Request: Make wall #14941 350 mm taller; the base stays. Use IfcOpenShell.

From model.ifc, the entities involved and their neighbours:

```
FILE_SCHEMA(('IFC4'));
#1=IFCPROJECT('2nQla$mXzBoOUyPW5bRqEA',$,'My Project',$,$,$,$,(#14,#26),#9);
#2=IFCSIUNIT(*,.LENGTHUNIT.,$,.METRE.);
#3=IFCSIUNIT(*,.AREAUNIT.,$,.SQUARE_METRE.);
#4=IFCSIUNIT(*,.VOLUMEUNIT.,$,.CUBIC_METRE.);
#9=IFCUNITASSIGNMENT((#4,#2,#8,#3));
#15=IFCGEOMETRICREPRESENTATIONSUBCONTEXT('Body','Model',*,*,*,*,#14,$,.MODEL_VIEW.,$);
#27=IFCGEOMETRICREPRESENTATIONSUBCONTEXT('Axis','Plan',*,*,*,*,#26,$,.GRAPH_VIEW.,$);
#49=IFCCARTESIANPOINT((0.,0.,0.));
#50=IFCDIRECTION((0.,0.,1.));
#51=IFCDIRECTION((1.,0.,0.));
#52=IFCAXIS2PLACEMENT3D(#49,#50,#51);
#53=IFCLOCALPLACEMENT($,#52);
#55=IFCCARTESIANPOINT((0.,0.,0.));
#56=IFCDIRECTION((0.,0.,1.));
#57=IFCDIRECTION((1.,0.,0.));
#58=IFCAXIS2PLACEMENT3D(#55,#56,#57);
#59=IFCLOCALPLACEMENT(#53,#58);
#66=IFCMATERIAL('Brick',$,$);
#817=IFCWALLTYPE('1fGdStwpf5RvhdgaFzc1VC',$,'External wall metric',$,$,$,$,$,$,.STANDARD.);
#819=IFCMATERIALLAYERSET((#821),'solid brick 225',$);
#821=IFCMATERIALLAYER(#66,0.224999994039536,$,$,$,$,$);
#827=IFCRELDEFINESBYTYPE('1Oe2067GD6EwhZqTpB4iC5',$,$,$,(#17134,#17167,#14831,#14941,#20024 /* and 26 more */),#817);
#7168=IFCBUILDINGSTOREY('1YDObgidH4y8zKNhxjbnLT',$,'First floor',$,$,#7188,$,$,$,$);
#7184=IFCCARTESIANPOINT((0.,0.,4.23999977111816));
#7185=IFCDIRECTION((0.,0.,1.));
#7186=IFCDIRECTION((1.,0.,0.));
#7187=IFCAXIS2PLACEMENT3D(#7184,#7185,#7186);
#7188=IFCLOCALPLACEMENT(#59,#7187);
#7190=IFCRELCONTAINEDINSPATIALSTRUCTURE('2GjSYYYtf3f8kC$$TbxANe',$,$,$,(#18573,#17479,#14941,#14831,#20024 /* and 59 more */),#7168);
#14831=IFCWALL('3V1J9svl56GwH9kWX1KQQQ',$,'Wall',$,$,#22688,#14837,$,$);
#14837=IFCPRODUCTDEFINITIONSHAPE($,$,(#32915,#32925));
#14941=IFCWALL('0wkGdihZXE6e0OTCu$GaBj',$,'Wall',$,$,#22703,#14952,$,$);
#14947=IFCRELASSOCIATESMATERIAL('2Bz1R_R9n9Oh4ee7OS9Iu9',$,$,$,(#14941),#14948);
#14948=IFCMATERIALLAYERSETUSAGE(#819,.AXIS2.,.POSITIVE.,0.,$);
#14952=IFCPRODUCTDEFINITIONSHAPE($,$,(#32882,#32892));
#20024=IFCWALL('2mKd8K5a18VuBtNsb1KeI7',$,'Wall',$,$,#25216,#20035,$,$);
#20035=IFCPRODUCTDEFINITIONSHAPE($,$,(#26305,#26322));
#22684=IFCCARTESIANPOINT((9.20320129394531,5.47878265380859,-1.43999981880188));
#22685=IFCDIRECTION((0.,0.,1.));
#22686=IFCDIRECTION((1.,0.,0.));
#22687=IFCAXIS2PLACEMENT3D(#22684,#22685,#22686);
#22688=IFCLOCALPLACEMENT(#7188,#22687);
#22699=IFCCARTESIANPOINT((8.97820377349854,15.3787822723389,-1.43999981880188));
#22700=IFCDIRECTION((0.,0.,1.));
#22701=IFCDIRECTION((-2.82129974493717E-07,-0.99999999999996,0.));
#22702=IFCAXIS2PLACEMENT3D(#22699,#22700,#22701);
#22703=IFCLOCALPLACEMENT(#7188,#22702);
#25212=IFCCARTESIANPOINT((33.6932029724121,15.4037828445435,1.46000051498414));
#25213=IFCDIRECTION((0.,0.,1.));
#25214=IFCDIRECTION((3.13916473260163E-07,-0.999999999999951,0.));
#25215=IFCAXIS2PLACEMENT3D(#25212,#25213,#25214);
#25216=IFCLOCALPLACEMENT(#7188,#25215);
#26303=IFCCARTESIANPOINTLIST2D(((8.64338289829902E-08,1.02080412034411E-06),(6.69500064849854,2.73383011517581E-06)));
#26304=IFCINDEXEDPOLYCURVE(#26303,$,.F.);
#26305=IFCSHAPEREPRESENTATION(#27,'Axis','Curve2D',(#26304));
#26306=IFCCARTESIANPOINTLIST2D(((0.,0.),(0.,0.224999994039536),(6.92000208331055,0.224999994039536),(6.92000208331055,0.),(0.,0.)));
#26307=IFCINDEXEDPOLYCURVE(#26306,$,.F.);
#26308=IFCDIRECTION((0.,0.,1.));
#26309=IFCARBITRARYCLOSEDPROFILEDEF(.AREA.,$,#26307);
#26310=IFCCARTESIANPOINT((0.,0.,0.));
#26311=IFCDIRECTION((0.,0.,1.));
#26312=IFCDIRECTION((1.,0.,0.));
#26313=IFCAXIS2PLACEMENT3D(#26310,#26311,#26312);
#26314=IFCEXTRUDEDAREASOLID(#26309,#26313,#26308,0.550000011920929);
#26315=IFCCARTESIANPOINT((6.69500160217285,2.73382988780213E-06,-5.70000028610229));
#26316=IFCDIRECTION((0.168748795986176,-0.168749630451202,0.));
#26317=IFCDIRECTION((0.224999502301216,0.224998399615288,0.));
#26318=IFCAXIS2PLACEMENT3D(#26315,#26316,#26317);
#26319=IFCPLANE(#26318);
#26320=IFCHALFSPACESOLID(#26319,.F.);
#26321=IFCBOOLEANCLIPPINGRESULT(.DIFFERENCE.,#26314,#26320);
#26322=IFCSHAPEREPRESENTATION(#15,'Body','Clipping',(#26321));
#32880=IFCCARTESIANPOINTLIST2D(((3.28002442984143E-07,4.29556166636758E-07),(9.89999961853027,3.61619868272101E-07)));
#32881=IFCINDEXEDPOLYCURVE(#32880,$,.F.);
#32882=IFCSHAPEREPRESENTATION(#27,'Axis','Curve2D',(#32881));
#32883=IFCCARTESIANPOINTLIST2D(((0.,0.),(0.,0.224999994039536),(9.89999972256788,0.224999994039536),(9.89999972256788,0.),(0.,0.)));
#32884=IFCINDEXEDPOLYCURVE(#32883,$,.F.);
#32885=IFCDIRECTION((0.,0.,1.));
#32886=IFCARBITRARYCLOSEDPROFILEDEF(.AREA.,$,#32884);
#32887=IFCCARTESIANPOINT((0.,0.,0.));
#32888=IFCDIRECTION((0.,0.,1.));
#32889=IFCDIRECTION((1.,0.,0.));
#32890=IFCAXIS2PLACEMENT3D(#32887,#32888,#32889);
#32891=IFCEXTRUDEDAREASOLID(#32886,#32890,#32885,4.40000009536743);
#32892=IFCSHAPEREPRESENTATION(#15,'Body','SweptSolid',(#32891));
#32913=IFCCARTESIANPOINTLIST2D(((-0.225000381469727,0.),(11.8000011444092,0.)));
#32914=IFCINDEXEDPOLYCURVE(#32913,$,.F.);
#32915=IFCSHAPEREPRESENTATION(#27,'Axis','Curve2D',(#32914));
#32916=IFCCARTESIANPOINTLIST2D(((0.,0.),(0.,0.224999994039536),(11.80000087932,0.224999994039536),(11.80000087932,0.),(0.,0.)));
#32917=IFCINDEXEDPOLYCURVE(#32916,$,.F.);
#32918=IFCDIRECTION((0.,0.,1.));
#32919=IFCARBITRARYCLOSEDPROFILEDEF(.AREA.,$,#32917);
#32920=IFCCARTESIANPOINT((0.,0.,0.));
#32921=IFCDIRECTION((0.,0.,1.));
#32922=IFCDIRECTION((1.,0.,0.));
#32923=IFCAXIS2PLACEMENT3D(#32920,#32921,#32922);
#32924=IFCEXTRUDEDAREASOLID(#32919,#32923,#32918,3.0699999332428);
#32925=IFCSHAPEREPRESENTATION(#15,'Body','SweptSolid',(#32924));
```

```python
import ifcopenshell
import ifcopenshell.geom
import ifcopenshell.util.representation
import ifcopenshell.util.shape
import ifcopenshell.util.unit

model = ifcopenshell.open("model.ifc")
unit_scale = ifcopenshell.util.unit.calculate_unit_scale(model)
settings = ifcopenshell.geom.settings()


def volume(element):
    """Net volume in cubic metres, openings subtracted."""
    shape = ifcopenshell.geom.create_shape(settings, element)
    return ifcopenshell.util.shape.get_volume(shape.geometry)


wall = model.by_guid("0wkGdihZXE6e0OTCu$GaBj")
before = volume(wall)

body = ifcopenshell.util.representation.get_representation(wall, "Model", "Body")
solid = body.Items[0]
old_height = solid.Depth
solid.Depth += 0.35 / unit_scale
after = volume(wall)

print(f"height {old_height:g} -> {solid.Depth:g}, volume {before:.3f} -> {after:.3f} m3")

model.write("model_rev.ifc")
```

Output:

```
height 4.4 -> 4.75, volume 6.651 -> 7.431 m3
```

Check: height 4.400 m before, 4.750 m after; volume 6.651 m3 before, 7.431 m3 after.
